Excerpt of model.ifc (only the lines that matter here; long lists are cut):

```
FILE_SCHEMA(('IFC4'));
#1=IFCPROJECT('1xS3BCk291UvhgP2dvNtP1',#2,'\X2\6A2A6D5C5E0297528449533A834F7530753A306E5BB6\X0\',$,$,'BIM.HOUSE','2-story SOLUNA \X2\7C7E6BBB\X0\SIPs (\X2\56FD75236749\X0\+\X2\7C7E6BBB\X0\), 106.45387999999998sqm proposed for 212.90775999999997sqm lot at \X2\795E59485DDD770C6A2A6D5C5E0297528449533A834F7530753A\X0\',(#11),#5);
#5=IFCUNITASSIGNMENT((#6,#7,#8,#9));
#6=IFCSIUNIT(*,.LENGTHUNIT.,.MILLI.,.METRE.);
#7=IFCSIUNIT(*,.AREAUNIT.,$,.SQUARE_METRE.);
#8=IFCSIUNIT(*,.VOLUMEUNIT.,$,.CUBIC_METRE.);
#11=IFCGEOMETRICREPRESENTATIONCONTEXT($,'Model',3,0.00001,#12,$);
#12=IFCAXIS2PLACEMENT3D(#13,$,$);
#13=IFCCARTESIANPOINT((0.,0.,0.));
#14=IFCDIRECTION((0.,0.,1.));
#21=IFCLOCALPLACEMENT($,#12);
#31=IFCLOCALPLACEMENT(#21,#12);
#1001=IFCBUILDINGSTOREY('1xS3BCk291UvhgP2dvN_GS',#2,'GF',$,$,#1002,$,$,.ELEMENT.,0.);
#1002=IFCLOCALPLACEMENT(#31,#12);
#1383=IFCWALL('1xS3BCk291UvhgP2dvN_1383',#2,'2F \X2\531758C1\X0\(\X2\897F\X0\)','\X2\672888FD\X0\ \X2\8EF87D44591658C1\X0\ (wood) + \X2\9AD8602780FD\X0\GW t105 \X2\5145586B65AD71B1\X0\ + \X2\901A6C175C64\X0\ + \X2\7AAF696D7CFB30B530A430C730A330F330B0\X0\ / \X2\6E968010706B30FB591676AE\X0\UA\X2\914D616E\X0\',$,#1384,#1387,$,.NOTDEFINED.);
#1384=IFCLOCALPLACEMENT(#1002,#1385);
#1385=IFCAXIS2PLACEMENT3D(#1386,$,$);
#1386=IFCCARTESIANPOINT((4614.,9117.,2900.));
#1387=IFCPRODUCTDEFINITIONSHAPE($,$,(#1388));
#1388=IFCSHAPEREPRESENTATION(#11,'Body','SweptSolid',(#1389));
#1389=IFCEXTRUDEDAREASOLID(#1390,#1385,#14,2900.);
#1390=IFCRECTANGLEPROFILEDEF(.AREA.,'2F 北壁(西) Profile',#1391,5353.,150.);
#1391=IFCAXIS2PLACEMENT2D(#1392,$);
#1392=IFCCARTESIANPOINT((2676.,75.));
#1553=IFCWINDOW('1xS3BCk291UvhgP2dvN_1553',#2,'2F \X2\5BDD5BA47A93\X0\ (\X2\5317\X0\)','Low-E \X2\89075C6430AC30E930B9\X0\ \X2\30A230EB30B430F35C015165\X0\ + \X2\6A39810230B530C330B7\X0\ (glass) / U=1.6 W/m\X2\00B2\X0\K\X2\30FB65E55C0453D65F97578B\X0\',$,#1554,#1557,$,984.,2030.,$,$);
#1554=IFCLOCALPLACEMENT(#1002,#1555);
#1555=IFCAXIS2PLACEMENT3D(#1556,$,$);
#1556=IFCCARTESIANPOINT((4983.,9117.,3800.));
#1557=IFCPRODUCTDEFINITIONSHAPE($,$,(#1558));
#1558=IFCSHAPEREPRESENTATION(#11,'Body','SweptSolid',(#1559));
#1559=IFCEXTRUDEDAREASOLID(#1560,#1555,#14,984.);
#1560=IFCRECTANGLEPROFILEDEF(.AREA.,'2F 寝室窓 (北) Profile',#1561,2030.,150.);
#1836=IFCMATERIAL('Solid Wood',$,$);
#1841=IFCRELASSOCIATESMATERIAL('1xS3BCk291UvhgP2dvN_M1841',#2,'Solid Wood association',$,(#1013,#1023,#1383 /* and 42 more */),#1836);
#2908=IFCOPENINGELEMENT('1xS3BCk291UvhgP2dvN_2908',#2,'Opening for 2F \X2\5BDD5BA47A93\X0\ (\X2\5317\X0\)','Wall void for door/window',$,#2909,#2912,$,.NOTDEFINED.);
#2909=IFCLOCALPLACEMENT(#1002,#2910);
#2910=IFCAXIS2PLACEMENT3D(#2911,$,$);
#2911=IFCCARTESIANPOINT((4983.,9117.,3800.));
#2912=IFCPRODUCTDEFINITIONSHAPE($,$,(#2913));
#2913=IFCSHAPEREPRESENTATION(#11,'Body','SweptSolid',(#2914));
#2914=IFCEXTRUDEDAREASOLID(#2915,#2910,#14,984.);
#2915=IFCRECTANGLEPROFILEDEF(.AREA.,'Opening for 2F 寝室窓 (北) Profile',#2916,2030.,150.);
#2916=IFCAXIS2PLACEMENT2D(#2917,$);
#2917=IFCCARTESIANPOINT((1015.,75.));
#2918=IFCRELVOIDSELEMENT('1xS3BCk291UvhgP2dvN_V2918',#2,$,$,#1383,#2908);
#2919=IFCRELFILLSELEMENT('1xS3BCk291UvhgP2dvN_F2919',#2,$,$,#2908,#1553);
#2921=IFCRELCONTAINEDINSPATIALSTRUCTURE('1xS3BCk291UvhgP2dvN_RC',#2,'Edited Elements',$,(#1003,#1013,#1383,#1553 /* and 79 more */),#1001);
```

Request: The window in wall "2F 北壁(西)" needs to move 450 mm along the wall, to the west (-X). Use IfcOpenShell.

```python
import ifcopenshell
import ifcopenshell.api.geometry
import ifcopenshell.util.placement
import ifcopenshell.util.unit

model = ifcopenshell.open("model.ifc")
unit_scale = ifcopenshell.util.unit.calculate_unit_scale(model)

window = model.by_guid("1xS3BCk291UvhgP2dvN_1553")
opening = window.FillsVoids[0].RelatingOpeningElement
wall = opening.VoidsElements[0].RelatingBuildingElement

wall_matrix = ifcopenshell.util.placement.get_local_placement(wall.ObjectPlacement)
shift = wall_matrix[:3, 0] * -0.45 / unit_scale
before = ifcopenshell.util.placement.get_local_placement(window.ObjectPlacement)[:3, 3].copy()

# The window is not placed relative to its opening, so move both.
for product in (opening, window):
    matrix = ifcopenshell.util.placement.get_local_placement(product.ObjectPlacement)
    matrix[:3, 3] += shift
    ifcopenshell.api.geometry.edit_object_placement(model, product=product, matrix=matrix, is_si=False)

after = ifcopenshell.util.placement.get_local_placement(window.ObjectPlacement)[:3, 3]
print("window moved by", (after - before).round(3) + 0.0)

model.write("model_edited.ifc")
```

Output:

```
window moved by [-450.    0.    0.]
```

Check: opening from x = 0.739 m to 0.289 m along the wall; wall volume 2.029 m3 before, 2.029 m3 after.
